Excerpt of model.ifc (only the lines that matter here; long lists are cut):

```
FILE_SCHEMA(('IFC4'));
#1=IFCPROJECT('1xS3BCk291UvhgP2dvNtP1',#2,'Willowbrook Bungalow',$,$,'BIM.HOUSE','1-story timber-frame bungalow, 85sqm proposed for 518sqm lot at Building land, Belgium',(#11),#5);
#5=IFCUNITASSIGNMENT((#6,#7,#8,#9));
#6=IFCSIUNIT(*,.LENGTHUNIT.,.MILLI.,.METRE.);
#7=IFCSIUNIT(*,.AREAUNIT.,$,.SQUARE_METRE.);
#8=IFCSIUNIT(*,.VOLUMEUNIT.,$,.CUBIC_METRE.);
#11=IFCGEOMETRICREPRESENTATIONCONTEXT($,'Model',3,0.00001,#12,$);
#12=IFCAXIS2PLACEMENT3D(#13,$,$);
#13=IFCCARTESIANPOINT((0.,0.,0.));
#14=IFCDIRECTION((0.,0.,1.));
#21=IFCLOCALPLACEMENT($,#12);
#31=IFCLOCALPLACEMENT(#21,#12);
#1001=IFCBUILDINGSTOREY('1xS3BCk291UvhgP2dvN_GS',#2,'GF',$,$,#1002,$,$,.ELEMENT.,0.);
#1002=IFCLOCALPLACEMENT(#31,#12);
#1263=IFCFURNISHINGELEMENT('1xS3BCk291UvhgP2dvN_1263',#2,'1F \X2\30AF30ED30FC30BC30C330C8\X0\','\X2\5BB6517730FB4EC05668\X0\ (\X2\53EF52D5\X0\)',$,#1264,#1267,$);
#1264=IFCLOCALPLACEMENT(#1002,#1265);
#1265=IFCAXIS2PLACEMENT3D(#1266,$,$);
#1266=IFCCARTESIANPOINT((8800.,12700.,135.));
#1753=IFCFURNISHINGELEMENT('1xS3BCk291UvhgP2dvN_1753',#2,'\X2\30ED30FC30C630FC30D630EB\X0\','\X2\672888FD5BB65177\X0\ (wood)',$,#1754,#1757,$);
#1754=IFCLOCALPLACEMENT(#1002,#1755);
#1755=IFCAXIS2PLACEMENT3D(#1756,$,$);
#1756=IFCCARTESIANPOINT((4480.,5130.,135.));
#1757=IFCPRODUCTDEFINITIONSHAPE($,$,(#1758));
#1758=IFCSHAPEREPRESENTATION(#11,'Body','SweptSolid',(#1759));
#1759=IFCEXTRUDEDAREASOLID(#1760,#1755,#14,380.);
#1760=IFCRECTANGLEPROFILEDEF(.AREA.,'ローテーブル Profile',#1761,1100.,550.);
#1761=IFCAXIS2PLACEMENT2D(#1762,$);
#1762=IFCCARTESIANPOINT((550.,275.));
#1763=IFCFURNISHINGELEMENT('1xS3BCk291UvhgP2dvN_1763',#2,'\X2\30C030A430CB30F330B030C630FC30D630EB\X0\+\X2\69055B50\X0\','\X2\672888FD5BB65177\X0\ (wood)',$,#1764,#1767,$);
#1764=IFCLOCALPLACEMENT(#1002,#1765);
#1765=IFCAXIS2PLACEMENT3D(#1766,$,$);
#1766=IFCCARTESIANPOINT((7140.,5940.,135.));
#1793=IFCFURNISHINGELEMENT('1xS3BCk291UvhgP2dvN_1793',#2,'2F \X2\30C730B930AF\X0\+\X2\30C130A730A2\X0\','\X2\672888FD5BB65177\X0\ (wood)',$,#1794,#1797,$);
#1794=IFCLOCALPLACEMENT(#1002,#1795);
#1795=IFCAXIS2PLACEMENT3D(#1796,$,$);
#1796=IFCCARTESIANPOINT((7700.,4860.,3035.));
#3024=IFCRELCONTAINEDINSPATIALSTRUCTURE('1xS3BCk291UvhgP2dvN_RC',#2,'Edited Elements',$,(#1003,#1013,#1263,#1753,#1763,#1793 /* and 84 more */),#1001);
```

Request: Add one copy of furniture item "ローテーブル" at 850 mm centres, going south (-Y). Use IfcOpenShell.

```python
import numpy as np
import ifcopenshell
import ifcopenshell.api.geometry
import ifcopenshell.api.root
import ifcopenshell.util.element
import ifcopenshell.util.placement
import ifcopenshell.util.unit

model = ifcopenshell.open("model.ifc")
unit_scale = ifcopenshell.util.unit.calculate_unit_scale(model)


def reuse_history(source, copy):
    """copy_class also copies each property set's owner history, people and application; keep the originals."""
    for rel in copy.IsDefinedBy:
        if rel.is_a("IfcRelDefinesByProperties") and (history := rel.RelatingPropertyDefinition.OwnerHistory):
            rel.RelatingPropertyDefinition.OwnerHistory = source.OwnerHistory
            ifcopenshell.util.element.remove_deep2(model, history)


source = model.by_guid("1xS3BCk291UvhgP2dvN_1753")
base = ifcopenshell.util.placement.get_local_placement(source.ObjectPlacement)
step = np.array([0.0, -1.0, 0.0]) * 0.85 / unit_scale

for i in range(1, 2):
    copy = ifcopenshell.api.root.copy_class(model, product=source)
    copy.Representation = ifcopenshell.util.element.copy_deep(
        model, source.Representation, exclude=["IfcGeometricRepresentationContext", "IfcRepresentationMap"]
    )
    reuse_history(source, copy)
    matrix = base.copy()
    matrix[:3, 3] += i * step
    print("added at", matrix[:3, 3].round(3) + 0.0)
    ifcopenshell.api.geometry.edit_object_placement(model, product=copy, matrix=matrix, is_si=False)

model.write("model_updated.ifc")
```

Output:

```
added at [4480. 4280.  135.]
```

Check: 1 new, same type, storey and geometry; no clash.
